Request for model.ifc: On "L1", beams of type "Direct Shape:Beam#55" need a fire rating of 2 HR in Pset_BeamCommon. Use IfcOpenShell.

First a look at what the model holds.

```python
import ifcopenshell
import ifcopenshell.util.element

model = ifcopenshell.open("model.ifc")
print(model.schema)
storey = next(s for s in model.by_type("IfcBuildingStorey") if s.Name == "L1")
beams = [e for e in ifcopenshell.util.element.get_decomposition(storey) if e.is_a("IfcBeam")]
seen = {}
for e in beams:
    element_type = ifcopenshell.util.element.get_type(e)
    key = (element_type.Name if element_type != e and element_type else None, ifcopenshell.util.element.get_pset(e, "Pset_BeamCommon", "FireRating"))
    seen[key] = seen.get(key, 0) + 1
for (name, value), count in sorted(seen.items(), key=str):
    print(count, "x", name, "|", value)
```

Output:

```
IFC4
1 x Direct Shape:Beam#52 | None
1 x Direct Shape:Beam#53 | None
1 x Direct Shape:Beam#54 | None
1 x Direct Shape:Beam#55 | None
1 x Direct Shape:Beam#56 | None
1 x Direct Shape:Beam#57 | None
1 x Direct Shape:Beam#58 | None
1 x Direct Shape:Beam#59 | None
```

```python
import ifcopenshell
import ifcopenshell.api.pset
import ifcopenshell.util.element

model = ifcopenshell.open("model.ifc")

storey = next(s for s in model.by_type("IfcBuildingStorey") if s.Name == "L1")
beams = [e for e in ifcopenshell.util.element.get_decomposition(storey) if e.is_a("IfcBeam")]

count = 0
for e in beams:
    element_type = ifcopenshell.util.element.get_type(e)
    if element_type in (None, e) or element_type.Name != "Direct Shape:Beam#55":
        continue
    # add_pset returns the element's existing set when there is one.
    pset = ifcopenshell.api.pset.add_pset(model, product=e, name="Pset_BeamCommon")
    ifcopenshell.api.pset.edit_pset(model, pset=pset, properties={"FireRating": "2 HR"})
    count += 1

print(count, "beams updated")

model.write("model_updated.ifc")
```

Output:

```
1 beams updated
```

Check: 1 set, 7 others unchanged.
